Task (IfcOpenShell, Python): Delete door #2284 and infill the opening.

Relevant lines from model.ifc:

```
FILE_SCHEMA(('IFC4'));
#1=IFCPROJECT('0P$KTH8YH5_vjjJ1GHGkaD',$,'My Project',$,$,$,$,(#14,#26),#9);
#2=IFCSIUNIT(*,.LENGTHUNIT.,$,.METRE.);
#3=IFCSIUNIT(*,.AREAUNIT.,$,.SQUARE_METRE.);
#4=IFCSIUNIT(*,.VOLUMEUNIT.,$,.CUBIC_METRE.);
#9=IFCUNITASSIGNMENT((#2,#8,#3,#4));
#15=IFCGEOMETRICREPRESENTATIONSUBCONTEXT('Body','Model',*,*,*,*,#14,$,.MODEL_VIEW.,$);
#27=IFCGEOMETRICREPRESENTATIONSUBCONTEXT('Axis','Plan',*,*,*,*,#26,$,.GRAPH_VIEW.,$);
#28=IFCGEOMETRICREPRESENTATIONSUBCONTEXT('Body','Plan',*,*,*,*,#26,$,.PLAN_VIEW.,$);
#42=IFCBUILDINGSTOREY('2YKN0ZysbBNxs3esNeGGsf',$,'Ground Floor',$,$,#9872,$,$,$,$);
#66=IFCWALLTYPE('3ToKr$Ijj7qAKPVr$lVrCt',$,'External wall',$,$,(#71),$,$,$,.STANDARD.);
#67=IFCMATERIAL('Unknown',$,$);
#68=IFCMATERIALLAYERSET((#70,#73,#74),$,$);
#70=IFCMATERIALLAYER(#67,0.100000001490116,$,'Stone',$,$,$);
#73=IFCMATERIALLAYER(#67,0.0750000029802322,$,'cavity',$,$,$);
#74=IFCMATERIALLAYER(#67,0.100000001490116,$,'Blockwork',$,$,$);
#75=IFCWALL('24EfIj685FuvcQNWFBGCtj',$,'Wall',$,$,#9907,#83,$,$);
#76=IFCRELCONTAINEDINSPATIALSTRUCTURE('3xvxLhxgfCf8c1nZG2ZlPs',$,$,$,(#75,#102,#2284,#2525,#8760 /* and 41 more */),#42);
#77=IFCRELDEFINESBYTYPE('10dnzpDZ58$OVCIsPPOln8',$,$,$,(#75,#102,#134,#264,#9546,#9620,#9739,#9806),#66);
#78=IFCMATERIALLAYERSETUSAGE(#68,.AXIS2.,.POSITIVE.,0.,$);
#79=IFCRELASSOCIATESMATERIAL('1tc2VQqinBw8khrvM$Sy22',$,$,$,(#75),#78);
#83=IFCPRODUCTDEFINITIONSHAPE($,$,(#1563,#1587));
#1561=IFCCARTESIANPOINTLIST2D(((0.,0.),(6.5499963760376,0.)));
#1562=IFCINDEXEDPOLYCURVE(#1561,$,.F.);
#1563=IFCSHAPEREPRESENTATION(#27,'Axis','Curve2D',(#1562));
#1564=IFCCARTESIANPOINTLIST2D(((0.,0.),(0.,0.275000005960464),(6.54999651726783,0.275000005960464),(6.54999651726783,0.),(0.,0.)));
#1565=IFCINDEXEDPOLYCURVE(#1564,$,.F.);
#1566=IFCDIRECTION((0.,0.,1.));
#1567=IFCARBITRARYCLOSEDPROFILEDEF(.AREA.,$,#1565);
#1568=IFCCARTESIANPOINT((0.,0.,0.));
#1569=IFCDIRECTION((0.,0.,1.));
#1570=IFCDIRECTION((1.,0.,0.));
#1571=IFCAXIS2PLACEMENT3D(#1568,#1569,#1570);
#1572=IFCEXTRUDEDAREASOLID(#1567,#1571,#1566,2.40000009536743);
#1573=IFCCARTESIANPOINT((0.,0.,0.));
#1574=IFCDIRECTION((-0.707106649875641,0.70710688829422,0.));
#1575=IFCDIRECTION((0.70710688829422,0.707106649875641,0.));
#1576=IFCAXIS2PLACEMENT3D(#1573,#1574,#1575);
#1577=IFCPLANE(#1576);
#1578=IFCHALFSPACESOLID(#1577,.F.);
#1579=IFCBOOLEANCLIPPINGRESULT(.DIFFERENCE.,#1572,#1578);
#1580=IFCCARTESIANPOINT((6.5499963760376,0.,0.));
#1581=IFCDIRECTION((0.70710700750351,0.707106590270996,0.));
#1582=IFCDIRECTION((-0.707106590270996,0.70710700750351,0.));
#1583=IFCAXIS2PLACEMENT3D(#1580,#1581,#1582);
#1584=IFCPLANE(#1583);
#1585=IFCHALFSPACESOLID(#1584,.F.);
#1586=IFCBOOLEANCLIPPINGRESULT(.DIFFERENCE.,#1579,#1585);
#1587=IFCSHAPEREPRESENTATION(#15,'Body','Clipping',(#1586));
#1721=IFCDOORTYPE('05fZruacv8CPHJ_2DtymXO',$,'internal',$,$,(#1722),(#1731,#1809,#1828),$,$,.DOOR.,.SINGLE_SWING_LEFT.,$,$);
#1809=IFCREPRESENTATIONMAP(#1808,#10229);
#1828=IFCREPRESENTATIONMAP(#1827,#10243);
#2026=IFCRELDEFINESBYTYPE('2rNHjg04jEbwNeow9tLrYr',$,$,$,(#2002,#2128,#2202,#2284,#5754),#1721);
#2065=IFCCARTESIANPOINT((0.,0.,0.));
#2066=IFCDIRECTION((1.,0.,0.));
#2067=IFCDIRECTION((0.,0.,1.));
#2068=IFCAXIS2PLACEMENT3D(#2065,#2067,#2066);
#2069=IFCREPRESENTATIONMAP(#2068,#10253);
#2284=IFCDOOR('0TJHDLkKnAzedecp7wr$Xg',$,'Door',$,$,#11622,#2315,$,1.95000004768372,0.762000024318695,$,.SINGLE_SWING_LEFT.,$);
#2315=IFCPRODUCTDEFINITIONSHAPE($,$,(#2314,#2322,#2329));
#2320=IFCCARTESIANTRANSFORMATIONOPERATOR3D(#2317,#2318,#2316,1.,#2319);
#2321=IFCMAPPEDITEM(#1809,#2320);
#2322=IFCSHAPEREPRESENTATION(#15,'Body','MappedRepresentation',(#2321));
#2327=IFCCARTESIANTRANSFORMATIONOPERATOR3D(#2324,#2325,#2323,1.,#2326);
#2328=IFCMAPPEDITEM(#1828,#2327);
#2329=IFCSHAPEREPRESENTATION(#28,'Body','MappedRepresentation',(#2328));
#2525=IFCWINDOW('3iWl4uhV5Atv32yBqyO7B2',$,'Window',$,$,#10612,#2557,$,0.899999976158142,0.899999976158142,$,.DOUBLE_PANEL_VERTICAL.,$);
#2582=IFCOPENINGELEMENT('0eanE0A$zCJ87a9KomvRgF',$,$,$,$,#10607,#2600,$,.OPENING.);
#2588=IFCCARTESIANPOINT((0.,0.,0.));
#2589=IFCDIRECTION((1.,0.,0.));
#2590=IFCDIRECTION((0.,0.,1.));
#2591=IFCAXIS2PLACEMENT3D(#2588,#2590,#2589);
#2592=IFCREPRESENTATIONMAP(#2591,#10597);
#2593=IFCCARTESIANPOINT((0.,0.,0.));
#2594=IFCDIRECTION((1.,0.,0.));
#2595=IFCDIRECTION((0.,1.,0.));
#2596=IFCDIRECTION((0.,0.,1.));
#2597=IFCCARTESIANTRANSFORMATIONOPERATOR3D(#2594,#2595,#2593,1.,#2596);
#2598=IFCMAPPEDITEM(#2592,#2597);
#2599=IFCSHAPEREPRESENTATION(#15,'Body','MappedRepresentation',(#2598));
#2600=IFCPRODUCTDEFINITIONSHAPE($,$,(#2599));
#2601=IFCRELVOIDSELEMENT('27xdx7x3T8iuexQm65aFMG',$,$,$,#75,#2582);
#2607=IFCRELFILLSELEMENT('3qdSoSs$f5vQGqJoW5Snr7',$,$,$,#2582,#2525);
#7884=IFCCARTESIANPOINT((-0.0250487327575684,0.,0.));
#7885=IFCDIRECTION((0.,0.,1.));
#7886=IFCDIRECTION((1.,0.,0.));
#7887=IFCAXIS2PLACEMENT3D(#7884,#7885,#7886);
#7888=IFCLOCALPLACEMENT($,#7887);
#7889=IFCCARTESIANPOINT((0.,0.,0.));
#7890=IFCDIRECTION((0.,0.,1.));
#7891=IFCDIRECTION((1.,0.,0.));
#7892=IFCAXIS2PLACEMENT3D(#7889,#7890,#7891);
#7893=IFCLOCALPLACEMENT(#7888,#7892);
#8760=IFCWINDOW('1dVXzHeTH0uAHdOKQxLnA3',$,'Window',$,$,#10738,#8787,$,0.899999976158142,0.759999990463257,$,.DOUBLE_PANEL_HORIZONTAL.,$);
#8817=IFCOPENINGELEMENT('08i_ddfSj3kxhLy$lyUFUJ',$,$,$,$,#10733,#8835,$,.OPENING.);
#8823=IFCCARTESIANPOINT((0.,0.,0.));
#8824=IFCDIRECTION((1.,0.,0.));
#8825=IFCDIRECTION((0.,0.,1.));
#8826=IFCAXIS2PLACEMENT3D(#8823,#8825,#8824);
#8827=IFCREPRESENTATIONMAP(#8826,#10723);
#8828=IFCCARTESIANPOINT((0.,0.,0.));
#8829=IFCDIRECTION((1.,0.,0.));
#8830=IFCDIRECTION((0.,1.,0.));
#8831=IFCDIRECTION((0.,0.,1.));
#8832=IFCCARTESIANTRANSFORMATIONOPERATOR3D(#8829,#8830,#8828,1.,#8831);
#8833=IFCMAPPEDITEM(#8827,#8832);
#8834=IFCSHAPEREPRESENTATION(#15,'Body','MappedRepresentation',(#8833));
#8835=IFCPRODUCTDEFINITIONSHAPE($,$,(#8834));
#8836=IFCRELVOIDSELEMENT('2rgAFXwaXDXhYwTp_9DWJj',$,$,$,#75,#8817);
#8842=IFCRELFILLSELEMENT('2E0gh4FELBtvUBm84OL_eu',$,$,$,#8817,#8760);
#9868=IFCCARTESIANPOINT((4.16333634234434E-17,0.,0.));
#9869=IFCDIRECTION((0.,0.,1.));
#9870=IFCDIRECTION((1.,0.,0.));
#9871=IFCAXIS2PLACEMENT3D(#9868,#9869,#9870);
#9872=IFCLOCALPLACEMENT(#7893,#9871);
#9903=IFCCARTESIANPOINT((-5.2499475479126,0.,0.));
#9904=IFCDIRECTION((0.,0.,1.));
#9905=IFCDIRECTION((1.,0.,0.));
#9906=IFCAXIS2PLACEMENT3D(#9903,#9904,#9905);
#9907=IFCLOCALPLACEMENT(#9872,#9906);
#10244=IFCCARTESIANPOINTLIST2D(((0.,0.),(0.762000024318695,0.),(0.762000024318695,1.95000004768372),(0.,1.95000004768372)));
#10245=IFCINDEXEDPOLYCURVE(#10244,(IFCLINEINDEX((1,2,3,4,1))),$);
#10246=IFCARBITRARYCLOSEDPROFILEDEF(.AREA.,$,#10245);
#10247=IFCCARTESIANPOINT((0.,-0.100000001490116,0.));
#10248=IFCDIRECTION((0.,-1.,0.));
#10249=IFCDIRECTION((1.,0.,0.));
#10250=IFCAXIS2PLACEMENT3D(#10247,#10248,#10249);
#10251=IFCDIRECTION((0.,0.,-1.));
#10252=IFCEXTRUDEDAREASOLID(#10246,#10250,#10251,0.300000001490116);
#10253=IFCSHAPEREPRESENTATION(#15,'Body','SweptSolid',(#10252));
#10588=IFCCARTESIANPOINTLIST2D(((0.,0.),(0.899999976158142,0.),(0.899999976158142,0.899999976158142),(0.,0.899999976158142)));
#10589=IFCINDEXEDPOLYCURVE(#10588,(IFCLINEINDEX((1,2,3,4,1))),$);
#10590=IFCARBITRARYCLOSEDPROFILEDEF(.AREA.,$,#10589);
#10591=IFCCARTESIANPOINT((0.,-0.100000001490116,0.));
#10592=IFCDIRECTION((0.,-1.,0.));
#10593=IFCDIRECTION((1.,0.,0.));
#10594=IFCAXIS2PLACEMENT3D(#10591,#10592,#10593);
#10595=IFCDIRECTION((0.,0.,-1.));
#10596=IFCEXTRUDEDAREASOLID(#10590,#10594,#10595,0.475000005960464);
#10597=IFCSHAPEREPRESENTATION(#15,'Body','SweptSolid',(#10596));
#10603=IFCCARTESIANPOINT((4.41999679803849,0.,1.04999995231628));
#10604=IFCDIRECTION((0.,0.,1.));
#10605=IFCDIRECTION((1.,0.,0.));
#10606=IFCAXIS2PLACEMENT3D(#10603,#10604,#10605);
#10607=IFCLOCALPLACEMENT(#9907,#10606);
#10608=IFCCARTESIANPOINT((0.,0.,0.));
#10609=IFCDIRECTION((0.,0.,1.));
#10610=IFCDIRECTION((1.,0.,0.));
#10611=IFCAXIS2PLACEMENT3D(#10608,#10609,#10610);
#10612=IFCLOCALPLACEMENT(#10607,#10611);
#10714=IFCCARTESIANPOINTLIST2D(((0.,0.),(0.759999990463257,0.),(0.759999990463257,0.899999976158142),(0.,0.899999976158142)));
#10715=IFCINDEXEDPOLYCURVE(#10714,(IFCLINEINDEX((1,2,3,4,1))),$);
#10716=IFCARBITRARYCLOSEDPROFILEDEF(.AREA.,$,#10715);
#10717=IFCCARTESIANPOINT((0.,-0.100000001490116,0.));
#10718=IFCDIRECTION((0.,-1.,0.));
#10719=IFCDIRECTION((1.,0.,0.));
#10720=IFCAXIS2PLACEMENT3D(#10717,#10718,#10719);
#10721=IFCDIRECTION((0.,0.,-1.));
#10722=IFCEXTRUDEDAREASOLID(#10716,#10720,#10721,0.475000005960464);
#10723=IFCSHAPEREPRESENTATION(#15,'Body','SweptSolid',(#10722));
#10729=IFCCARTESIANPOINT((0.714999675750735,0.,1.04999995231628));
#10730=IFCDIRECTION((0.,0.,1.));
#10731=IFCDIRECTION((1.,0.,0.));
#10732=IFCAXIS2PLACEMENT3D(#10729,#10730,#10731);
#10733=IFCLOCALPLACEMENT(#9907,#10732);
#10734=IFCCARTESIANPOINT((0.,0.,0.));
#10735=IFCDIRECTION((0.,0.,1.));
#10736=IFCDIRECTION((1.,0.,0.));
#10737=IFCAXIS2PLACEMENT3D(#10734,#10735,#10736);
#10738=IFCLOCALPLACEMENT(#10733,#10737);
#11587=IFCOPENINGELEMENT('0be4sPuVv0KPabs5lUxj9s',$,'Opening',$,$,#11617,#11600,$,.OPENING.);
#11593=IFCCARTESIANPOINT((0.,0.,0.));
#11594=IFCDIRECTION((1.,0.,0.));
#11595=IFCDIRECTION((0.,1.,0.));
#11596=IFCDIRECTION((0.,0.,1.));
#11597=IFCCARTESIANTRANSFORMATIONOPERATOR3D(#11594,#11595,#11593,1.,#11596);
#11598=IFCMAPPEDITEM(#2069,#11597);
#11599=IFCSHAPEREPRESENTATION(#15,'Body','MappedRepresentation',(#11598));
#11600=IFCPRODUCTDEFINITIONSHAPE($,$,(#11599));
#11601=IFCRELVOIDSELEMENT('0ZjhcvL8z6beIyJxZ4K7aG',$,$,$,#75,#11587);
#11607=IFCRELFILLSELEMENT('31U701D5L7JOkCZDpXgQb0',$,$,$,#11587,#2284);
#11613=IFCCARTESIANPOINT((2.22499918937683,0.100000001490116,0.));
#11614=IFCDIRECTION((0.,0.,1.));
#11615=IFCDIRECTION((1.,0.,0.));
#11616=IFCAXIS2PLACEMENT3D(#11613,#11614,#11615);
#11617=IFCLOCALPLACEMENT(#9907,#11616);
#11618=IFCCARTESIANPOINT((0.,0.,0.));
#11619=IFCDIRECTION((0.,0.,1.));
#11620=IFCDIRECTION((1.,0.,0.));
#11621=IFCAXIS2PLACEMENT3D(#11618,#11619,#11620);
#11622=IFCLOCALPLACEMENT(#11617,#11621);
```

```python
import ifcopenshell
import ifcopenshell.api.feature
import ifcopenshell.api.root
import ifcopenshell.geom
import ifcopenshell.util.shape

model = ifcopenshell.open("model.ifc")
settings = ifcopenshell.geom.settings()


def volume(element):
    """Net volume in cubic metres, openings subtracted."""
    shape = ifcopenshell.geom.create_shape(settings, element)
    return ifcopenshell.util.shape.get_volume(shape.geometry)


door = model.by_guid("0TJHDLkKnAzedecp7wr$Xg")
opening = door.FillsVoids[0].RelatingOpeningElement
wall = opening.VoidsElements[0].RelatingBuildingElement
before = volume(wall)

ifcopenshell.api.root.remove_product(model, product=door)
ifcopenshell.api.feature.remove_feature(model, feature=opening)

after = volume(wall)

print(f"wall volume {before:.3f} -> {after:.3f} m3")

model.write("model_updated.ifc")
```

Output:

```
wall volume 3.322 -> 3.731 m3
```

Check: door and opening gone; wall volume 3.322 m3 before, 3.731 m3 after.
